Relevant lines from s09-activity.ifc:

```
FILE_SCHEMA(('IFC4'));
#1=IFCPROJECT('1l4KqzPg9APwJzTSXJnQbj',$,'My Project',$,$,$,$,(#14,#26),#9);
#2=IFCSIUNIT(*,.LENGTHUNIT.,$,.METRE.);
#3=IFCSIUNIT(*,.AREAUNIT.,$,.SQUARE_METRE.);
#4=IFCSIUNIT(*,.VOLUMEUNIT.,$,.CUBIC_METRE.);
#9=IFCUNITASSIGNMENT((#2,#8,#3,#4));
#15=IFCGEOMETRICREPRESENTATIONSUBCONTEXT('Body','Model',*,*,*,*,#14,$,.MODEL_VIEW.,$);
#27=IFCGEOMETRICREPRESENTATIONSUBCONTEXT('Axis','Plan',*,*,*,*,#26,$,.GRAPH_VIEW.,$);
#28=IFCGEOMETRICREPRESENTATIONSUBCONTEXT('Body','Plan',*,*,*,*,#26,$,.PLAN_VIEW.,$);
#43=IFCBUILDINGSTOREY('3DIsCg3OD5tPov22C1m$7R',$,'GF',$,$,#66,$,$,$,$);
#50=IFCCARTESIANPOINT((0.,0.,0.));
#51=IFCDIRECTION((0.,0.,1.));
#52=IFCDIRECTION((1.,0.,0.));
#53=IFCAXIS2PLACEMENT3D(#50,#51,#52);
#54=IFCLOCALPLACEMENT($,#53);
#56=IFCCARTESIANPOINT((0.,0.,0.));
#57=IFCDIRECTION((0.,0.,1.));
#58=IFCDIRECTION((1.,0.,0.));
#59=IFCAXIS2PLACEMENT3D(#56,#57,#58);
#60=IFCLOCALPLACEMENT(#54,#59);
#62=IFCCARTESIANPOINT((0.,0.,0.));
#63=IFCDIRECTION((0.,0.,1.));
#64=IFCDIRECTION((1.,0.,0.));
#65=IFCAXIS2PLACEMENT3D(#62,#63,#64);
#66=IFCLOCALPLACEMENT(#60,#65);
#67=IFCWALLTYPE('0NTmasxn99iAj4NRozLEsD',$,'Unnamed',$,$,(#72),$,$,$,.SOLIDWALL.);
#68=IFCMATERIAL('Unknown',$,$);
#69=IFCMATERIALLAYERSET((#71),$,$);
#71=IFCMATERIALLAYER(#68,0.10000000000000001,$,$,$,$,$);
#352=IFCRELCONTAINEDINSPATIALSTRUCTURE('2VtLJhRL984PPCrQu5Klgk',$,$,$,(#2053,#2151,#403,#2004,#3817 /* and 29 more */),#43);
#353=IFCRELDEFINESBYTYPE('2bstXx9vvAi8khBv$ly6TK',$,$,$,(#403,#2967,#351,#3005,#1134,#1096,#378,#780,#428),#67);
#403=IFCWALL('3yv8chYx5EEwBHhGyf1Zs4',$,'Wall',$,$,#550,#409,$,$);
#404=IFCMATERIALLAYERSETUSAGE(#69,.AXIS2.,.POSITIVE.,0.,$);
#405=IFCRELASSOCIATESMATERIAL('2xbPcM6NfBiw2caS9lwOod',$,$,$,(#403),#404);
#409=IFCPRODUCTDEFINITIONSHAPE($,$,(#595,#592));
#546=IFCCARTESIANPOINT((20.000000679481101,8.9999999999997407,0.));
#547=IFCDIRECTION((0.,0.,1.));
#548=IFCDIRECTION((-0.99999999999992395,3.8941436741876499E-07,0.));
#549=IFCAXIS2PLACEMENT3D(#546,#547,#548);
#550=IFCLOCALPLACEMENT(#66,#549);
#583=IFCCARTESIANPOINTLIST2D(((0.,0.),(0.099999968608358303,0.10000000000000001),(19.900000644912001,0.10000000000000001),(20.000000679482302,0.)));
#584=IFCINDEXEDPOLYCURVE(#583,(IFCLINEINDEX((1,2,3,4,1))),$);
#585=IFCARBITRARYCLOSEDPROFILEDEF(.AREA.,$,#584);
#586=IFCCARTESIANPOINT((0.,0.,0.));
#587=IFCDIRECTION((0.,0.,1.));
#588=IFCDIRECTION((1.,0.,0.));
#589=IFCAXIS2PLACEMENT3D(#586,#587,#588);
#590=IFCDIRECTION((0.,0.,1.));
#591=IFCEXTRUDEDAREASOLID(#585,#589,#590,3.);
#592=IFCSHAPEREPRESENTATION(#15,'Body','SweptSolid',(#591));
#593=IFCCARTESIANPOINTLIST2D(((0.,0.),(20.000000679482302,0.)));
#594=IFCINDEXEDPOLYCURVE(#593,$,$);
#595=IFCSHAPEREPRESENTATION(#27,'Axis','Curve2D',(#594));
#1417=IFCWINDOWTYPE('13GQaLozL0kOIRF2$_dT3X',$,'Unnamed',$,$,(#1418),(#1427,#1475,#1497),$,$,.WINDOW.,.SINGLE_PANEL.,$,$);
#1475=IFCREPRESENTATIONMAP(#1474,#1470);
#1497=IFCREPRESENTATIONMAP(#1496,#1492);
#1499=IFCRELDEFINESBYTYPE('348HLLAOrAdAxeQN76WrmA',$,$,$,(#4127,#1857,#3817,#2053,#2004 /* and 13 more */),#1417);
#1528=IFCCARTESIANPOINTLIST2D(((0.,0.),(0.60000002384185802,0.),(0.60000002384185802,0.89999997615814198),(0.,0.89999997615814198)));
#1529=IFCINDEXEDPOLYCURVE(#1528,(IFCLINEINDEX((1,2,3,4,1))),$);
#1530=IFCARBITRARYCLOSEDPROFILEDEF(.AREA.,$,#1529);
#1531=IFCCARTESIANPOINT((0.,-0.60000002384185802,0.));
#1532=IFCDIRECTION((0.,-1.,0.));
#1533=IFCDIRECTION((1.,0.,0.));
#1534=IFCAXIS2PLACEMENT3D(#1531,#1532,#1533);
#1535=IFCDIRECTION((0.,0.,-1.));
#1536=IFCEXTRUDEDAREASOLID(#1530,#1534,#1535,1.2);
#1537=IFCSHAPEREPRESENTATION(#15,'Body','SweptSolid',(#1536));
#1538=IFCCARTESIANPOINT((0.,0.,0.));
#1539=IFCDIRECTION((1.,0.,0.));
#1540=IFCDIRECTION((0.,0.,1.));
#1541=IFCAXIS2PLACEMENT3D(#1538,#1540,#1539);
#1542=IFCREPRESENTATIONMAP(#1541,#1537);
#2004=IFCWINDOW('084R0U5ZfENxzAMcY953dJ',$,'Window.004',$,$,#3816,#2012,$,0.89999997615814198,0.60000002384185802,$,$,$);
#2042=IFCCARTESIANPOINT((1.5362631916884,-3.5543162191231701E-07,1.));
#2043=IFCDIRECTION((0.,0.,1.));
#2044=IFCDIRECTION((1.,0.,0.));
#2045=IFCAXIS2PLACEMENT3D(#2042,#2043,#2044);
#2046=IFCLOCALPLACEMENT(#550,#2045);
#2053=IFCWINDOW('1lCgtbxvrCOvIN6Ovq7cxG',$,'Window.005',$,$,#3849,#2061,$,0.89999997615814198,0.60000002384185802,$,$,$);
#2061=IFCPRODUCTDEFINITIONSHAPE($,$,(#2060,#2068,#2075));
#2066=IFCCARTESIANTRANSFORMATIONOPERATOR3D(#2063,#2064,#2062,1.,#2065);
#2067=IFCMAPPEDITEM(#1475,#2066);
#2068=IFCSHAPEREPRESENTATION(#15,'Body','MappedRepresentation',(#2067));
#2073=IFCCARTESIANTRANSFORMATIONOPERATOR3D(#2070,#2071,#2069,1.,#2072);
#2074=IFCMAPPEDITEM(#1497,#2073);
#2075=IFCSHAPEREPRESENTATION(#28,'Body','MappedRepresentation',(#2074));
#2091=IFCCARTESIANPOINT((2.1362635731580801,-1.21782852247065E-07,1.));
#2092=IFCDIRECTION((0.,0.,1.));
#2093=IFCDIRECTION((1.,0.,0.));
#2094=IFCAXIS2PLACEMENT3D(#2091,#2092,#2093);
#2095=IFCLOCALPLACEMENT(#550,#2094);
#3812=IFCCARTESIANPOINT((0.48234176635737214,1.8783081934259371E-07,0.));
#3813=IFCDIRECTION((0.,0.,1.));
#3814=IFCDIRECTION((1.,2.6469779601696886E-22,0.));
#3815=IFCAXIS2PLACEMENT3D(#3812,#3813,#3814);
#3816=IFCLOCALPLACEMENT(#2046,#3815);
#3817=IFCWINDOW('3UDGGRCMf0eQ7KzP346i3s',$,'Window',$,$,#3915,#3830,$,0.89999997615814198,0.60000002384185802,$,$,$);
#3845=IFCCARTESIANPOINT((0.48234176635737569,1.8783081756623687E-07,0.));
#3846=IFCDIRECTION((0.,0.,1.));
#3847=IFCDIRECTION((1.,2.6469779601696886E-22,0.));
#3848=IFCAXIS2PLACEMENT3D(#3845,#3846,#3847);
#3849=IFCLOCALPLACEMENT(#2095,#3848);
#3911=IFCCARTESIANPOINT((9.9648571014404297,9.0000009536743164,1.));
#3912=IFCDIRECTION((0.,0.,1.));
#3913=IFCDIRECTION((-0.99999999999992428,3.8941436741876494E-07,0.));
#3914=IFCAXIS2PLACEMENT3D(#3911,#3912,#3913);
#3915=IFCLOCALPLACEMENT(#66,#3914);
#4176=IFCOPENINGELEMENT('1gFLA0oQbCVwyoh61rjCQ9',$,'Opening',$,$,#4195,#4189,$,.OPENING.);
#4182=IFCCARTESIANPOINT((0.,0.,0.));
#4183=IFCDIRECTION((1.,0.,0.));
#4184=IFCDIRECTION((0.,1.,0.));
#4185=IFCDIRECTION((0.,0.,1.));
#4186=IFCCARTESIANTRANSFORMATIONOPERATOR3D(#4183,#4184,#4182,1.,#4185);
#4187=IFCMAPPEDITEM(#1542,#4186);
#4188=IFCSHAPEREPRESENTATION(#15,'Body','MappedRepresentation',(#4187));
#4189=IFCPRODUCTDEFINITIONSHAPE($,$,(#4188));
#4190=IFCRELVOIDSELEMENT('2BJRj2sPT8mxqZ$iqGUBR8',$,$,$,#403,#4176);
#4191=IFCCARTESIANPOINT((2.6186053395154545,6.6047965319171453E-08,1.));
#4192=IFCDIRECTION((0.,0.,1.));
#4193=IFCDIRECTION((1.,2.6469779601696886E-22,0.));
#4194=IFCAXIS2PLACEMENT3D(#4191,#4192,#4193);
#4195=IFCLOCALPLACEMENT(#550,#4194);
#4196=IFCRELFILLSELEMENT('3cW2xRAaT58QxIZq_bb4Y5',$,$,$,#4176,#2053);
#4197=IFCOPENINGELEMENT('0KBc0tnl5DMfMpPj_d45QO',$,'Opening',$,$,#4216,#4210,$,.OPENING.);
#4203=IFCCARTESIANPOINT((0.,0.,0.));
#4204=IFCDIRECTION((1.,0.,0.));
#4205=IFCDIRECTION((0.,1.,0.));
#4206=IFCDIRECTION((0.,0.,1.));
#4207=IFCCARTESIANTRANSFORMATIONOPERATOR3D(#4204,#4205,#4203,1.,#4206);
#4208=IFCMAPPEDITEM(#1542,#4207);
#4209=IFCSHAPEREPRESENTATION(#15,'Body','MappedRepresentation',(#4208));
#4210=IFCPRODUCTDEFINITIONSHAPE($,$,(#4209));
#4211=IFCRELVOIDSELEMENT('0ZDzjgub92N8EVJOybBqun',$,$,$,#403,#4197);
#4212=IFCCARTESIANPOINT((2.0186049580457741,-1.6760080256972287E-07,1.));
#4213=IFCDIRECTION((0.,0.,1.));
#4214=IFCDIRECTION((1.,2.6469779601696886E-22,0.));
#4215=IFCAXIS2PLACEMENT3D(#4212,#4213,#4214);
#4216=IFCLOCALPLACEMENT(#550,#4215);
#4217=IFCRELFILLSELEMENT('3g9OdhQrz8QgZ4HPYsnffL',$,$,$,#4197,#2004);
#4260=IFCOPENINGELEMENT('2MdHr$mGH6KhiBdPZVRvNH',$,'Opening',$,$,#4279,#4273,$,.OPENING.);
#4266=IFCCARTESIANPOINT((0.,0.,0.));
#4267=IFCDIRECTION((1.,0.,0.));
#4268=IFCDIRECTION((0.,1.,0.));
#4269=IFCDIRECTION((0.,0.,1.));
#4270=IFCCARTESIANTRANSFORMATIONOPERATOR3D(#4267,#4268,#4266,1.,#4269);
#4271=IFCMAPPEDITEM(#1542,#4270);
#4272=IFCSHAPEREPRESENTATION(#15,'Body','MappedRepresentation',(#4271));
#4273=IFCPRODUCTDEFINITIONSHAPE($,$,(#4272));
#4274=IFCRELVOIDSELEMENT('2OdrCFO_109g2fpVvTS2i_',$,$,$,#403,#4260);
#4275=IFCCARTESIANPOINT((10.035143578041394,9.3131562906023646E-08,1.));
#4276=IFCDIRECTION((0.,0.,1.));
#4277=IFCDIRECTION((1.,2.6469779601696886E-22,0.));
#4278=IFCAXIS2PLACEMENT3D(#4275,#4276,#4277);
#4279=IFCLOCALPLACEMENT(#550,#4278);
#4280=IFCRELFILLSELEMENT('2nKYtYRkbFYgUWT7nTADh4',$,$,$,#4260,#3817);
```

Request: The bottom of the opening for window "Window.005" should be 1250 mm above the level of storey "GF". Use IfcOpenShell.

```python
import numpy as np
import ifcopenshell
import ifcopenshell.api.geometry
import ifcopenshell.geom
import ifcopenshell.util.element
import ifcopenshell.util.placement
import ifcopenshell.util.shape
import ifcopenshell.util.unit

model = ifcopenshell.open("s09-activity.ifc")
unit_scale = ifcopenshell.util.unit.calculate_unit_scale(model)

window = model.by_guid("1lCgtbxvrCOvIN6Ovq7cxG")
opening = window.FillsVoids[0].RelatingOpeningElement
storey = ifcopenshell.util.element.get_container(window, ifc_class="IfcBuildingStorey")
level = ifcopenshell.util.placement.get_local_placement(storey.ObjectPlacement)[2, 3]

# The opening's origin need not be at the sill, so measure its lowest point.
shape = ifcopenshell.geom.create_shape(ifcopenshell.geom.settings(), opening)
bottom = ifcopenshell.util.shape.get_shape_bottom_elevation(shape, shape.geometry) / unit_scale
dz = level + 1.25 - bottom

shift = np.array([0.0, 0.0, dz])
# The window is not placed relative to its opening, so move both.
for product in (opening, window):
    matrix = ifcopenshell.util.placement.get_local_placement(product.ObjectPlacement)
    matrix[:3, 3] += shift
    ifcopenshell.api.geometry.edit_object_placement(model, product=product, matrix=matrix, is_si=False)

print(f"moved by {dz * unit_scale:+.3f} m")

model.write("s09-activity_updated.ifc")
```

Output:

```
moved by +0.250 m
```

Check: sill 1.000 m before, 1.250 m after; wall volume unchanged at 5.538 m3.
